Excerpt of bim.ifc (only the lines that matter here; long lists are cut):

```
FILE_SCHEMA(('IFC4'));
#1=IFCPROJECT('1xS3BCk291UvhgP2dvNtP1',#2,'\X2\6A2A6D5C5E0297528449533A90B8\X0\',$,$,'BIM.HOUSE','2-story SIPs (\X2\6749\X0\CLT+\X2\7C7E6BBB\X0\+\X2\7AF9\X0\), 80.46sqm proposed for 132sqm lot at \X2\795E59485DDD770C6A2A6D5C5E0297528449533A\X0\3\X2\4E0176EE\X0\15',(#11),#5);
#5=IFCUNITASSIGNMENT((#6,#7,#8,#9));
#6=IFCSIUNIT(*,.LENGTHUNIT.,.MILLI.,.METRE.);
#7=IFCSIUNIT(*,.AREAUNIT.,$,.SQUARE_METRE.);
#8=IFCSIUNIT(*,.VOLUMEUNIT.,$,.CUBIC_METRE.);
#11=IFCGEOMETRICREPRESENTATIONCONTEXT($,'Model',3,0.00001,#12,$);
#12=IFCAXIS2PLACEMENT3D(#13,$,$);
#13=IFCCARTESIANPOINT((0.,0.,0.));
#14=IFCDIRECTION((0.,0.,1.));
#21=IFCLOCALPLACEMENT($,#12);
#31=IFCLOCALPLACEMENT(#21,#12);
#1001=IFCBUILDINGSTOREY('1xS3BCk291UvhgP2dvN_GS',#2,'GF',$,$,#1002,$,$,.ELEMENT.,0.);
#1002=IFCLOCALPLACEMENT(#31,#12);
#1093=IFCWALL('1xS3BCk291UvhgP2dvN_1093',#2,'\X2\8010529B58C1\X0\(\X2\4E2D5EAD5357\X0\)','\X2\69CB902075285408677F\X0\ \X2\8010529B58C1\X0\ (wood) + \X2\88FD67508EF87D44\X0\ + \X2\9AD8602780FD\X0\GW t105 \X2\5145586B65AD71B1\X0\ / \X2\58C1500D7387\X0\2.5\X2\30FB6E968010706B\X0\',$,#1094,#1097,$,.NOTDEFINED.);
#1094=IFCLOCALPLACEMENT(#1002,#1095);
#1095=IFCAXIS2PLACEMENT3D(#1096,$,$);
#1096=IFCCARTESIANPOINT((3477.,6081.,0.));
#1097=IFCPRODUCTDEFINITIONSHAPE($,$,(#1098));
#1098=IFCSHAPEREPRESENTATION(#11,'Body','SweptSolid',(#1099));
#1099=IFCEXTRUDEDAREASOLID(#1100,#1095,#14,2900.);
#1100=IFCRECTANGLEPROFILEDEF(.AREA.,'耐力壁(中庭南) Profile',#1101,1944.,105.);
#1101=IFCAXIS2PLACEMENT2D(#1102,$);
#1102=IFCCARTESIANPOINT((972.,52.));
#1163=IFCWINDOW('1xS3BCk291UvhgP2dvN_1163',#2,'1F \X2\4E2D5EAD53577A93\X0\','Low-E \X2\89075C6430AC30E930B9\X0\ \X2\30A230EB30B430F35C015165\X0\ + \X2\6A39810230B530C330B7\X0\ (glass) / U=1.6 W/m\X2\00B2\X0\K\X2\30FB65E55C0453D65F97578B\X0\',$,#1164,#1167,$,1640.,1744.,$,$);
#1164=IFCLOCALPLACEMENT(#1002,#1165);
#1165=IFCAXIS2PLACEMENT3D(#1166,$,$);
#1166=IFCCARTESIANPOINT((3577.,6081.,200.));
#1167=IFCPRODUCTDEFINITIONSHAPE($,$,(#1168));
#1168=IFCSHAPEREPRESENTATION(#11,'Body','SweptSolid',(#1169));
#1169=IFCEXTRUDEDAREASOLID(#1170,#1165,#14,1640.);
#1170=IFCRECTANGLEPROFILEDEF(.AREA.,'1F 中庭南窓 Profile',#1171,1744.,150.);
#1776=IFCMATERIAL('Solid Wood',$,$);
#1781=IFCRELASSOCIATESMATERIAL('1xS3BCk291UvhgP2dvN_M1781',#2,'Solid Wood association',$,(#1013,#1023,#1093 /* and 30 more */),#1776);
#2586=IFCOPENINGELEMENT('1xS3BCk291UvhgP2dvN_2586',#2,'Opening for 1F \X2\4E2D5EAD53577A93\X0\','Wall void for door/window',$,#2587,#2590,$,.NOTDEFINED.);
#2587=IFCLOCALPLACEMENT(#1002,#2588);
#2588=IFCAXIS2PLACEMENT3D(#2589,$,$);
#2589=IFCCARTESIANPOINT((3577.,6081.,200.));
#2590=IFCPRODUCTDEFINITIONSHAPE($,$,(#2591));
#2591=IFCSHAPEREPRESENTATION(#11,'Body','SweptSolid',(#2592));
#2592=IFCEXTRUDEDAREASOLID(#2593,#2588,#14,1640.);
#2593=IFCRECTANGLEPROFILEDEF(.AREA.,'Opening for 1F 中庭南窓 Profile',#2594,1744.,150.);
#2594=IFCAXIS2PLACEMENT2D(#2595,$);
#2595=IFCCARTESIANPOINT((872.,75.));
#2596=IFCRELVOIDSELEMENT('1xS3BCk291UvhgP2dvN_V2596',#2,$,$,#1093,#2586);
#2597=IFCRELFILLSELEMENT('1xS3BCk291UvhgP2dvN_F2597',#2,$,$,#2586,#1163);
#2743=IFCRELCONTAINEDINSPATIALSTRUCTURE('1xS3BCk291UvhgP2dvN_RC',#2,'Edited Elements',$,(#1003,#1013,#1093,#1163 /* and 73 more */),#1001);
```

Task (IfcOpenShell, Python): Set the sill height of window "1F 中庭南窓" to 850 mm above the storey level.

```python
import numpy as np
import ifcopenshell
import ifcopenshell.api.geometry
import ifcopenshell.geom
import ifcopenshell.util.element
import ifcopenshell.util.placement
import ifcopenshell.util.shape
import ifcopenshell.util.unit

model = ifcopenshell.open("bim.ifc")
unit_scale = ifcopenshell.util.unit.calculate_unit_scale(model)

window = model.by_id(1163)
opening = window.FillsVoids[0].RelatingOpeningElement
storey = ifcopenshell.util.element.get_container(window, ifc_class="IfcBuildingStorey")
level = ifcopenshell.util.placement.get_local_placement(storey.ObjectPlacement)[2, 3]

# The opening's origin need not be at the sill, so measure its lowest point.
shape = ifcopenshell.geom.create_shape(ifcopenshell.geom.settings(), opening)
bottom = ifcopenshell.util.shape.get_shape_bottom_elevation(shape, shape.geometry) / unit_scale
dz = level + 0.85 / unit_scale - bottom

shift = np.array([0.0, 0.0, dz])
# The window is not placed relative to its opening, so move both.
for product in (opening, window):
    matrix = ifcopenshell.util.placement.get_local_placement(product.ObjectPlacement)
    matrix[:3, 3] += shift
    ifcopenshell.api.geometry.edit_object_placement(model, product=product, matrix=matrix, is_si=False)

print(f"moved by {dz * unit_scale:+.3f} m")

model.write("bim_updated.ifc")
```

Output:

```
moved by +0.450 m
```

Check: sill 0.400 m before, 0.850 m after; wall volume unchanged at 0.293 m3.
